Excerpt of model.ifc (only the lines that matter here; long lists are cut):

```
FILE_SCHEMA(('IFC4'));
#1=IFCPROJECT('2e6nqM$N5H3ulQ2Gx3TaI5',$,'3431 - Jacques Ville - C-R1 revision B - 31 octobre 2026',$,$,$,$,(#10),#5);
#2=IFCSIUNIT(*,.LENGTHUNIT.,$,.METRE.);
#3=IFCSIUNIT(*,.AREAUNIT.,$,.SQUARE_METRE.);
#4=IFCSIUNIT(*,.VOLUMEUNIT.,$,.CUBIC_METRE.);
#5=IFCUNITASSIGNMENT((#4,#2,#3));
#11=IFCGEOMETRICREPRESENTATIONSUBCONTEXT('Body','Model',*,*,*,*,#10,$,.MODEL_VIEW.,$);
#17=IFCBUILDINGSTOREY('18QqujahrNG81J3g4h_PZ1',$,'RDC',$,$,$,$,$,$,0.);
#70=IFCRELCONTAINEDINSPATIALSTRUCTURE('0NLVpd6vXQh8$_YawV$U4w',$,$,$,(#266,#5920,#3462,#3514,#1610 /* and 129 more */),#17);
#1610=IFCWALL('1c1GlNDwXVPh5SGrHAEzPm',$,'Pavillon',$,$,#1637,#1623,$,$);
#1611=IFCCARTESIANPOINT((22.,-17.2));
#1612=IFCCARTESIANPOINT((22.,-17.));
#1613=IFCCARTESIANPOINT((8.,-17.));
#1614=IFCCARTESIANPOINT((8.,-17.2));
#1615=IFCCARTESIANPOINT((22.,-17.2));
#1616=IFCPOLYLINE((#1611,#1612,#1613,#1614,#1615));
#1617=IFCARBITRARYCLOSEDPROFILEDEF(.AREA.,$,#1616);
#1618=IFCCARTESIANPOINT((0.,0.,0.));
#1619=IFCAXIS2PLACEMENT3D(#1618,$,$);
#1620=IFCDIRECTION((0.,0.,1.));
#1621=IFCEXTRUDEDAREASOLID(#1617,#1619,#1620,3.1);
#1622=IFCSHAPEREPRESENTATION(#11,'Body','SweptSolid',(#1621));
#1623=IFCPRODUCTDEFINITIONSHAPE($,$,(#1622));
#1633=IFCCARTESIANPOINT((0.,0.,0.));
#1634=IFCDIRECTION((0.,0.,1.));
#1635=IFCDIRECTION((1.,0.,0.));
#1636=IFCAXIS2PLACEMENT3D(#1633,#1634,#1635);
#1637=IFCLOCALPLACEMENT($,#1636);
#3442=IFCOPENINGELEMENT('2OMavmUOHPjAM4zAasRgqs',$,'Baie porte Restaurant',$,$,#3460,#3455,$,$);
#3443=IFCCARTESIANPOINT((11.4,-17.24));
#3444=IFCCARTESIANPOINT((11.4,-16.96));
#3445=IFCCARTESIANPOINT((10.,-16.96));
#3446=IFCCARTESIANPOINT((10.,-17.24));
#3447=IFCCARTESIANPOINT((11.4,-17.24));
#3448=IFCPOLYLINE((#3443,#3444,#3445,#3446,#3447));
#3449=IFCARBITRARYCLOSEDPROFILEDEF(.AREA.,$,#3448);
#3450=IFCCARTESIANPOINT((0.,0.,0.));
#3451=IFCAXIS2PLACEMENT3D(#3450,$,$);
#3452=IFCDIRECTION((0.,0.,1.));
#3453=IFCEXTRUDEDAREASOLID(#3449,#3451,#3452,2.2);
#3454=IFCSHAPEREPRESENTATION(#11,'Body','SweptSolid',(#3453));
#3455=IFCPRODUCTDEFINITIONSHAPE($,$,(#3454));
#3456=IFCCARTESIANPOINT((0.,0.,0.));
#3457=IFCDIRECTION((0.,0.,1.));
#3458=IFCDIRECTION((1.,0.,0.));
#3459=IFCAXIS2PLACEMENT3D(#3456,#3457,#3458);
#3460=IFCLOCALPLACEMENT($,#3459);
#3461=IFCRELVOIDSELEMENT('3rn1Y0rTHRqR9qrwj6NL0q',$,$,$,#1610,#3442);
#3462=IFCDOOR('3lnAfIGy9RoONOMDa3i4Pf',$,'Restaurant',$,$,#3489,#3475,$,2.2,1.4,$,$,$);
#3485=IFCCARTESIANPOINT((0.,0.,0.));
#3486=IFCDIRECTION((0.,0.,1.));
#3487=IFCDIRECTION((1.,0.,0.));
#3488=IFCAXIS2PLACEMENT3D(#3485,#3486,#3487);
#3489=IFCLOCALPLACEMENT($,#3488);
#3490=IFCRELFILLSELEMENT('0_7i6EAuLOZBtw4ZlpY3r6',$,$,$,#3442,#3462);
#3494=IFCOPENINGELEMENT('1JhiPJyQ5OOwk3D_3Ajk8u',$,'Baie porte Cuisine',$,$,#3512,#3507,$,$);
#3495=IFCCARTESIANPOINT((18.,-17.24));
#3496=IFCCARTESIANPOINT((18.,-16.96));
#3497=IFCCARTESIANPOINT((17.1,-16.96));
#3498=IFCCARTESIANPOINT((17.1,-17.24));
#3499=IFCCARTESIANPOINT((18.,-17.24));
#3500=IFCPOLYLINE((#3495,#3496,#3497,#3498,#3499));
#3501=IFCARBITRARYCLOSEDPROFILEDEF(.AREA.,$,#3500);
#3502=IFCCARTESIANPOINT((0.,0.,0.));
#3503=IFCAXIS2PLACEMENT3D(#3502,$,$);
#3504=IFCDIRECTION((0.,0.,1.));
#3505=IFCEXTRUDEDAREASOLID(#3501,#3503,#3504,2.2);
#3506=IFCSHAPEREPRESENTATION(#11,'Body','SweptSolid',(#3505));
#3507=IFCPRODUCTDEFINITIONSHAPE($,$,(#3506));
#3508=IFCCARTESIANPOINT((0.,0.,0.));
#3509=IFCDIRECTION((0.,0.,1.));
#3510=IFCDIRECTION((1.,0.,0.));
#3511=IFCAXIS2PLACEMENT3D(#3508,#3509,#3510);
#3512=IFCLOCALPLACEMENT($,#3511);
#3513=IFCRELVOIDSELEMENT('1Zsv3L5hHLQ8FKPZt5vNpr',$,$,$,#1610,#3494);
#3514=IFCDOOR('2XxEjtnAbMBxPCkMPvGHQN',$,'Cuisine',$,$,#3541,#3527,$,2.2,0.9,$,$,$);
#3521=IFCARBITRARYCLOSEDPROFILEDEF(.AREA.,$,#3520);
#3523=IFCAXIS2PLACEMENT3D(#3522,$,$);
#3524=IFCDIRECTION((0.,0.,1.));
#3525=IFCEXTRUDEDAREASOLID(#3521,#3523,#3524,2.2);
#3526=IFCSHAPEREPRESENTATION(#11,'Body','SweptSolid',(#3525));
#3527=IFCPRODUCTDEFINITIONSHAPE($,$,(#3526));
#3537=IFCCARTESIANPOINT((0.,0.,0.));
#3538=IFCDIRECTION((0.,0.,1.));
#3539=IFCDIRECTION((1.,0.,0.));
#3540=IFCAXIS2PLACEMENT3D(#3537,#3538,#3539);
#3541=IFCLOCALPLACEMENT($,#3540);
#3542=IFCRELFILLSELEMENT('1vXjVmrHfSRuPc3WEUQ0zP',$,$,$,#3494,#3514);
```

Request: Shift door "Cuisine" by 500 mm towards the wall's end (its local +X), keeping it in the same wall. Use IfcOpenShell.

```python
import ifcopenshell
import ifcopenshell.api.geometry
import ifcopenshell.util.placement
import ifcopenshell.util.unit

model = ifcopenshell.open("model.ifc")
unit_scale = ifcopenshell.util.unit.calculate_unit_scale(model)

door = model.by_id(3514)
opening = door.FillsVoids[0].RelatingOpeningElement
wall = opening.VoidsElements[0].RelatingBuildingElement

wall_matrix = ifcopenshell.util.placement.get_local_placement(wall.ObjectPlacement)
shift = wall_matrix[:3, 0] * 0.5 / unit_scale
before = ifcopenshell.util.placement.get_local_placement(door.ObjectPlacement)[:3, 3].copy()

# The door is not placed relative to its opening, so move both.
for product in (opening, door):
    matrix = ifcopenshell.util.placement.get_local_placement(product.ObjectPlacement)
    matrix[:3, 3] += shift
    ifcopenshell.api.geometry.edit_object_placement(model, product=product, matrix=matrix, is_si=False)

after = ifcopenshell.util.placement.get_local_placement(door.ObjectPlacement)[:3, 3]
print("door moved by", (after - before).round(3) + 0.0)

model.write("model_rev.ifc")
```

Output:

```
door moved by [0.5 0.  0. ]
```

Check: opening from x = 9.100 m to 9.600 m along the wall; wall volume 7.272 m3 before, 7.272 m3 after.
